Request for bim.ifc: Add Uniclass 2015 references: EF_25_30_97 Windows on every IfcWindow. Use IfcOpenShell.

First a look at what the model holds.

```python
import ifcopenshell

model = ifcopenshell.open("bim.ifc")
print(model.schema)
print("classifications:", [c.Name for c in model.by_type("IfcClassification")])
for ifc_class in ("IfcDoor", "IfcRoof", "IfcStair", "IfcWall", "IfcWindow"):
    print(ifc_class, len(model.by_type(ifc_class)))
```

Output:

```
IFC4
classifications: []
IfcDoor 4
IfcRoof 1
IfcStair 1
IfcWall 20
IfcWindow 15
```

```python
import ifcopenshell
import ifcopenshell.api.classification

model = ifcopenshell.open("bim.ifc")

system = ifcopenshell.api.classification.add_classification(model, classification="Uniclass 2015")

codes = {
    "IfcWindow": ("EF_25_30_97", "Windows"),
}
for ifc_class, (code, name) in codes.items():
    products = model.by_type(ifc_class)
    ifcopenshell.api.classification.add_reference(
        model, products=products, classification=system, identification=code, name=name
    )
    print(code, len(products))

model.write("bim_rev.ifc")
```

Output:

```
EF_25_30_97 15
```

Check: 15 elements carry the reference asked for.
